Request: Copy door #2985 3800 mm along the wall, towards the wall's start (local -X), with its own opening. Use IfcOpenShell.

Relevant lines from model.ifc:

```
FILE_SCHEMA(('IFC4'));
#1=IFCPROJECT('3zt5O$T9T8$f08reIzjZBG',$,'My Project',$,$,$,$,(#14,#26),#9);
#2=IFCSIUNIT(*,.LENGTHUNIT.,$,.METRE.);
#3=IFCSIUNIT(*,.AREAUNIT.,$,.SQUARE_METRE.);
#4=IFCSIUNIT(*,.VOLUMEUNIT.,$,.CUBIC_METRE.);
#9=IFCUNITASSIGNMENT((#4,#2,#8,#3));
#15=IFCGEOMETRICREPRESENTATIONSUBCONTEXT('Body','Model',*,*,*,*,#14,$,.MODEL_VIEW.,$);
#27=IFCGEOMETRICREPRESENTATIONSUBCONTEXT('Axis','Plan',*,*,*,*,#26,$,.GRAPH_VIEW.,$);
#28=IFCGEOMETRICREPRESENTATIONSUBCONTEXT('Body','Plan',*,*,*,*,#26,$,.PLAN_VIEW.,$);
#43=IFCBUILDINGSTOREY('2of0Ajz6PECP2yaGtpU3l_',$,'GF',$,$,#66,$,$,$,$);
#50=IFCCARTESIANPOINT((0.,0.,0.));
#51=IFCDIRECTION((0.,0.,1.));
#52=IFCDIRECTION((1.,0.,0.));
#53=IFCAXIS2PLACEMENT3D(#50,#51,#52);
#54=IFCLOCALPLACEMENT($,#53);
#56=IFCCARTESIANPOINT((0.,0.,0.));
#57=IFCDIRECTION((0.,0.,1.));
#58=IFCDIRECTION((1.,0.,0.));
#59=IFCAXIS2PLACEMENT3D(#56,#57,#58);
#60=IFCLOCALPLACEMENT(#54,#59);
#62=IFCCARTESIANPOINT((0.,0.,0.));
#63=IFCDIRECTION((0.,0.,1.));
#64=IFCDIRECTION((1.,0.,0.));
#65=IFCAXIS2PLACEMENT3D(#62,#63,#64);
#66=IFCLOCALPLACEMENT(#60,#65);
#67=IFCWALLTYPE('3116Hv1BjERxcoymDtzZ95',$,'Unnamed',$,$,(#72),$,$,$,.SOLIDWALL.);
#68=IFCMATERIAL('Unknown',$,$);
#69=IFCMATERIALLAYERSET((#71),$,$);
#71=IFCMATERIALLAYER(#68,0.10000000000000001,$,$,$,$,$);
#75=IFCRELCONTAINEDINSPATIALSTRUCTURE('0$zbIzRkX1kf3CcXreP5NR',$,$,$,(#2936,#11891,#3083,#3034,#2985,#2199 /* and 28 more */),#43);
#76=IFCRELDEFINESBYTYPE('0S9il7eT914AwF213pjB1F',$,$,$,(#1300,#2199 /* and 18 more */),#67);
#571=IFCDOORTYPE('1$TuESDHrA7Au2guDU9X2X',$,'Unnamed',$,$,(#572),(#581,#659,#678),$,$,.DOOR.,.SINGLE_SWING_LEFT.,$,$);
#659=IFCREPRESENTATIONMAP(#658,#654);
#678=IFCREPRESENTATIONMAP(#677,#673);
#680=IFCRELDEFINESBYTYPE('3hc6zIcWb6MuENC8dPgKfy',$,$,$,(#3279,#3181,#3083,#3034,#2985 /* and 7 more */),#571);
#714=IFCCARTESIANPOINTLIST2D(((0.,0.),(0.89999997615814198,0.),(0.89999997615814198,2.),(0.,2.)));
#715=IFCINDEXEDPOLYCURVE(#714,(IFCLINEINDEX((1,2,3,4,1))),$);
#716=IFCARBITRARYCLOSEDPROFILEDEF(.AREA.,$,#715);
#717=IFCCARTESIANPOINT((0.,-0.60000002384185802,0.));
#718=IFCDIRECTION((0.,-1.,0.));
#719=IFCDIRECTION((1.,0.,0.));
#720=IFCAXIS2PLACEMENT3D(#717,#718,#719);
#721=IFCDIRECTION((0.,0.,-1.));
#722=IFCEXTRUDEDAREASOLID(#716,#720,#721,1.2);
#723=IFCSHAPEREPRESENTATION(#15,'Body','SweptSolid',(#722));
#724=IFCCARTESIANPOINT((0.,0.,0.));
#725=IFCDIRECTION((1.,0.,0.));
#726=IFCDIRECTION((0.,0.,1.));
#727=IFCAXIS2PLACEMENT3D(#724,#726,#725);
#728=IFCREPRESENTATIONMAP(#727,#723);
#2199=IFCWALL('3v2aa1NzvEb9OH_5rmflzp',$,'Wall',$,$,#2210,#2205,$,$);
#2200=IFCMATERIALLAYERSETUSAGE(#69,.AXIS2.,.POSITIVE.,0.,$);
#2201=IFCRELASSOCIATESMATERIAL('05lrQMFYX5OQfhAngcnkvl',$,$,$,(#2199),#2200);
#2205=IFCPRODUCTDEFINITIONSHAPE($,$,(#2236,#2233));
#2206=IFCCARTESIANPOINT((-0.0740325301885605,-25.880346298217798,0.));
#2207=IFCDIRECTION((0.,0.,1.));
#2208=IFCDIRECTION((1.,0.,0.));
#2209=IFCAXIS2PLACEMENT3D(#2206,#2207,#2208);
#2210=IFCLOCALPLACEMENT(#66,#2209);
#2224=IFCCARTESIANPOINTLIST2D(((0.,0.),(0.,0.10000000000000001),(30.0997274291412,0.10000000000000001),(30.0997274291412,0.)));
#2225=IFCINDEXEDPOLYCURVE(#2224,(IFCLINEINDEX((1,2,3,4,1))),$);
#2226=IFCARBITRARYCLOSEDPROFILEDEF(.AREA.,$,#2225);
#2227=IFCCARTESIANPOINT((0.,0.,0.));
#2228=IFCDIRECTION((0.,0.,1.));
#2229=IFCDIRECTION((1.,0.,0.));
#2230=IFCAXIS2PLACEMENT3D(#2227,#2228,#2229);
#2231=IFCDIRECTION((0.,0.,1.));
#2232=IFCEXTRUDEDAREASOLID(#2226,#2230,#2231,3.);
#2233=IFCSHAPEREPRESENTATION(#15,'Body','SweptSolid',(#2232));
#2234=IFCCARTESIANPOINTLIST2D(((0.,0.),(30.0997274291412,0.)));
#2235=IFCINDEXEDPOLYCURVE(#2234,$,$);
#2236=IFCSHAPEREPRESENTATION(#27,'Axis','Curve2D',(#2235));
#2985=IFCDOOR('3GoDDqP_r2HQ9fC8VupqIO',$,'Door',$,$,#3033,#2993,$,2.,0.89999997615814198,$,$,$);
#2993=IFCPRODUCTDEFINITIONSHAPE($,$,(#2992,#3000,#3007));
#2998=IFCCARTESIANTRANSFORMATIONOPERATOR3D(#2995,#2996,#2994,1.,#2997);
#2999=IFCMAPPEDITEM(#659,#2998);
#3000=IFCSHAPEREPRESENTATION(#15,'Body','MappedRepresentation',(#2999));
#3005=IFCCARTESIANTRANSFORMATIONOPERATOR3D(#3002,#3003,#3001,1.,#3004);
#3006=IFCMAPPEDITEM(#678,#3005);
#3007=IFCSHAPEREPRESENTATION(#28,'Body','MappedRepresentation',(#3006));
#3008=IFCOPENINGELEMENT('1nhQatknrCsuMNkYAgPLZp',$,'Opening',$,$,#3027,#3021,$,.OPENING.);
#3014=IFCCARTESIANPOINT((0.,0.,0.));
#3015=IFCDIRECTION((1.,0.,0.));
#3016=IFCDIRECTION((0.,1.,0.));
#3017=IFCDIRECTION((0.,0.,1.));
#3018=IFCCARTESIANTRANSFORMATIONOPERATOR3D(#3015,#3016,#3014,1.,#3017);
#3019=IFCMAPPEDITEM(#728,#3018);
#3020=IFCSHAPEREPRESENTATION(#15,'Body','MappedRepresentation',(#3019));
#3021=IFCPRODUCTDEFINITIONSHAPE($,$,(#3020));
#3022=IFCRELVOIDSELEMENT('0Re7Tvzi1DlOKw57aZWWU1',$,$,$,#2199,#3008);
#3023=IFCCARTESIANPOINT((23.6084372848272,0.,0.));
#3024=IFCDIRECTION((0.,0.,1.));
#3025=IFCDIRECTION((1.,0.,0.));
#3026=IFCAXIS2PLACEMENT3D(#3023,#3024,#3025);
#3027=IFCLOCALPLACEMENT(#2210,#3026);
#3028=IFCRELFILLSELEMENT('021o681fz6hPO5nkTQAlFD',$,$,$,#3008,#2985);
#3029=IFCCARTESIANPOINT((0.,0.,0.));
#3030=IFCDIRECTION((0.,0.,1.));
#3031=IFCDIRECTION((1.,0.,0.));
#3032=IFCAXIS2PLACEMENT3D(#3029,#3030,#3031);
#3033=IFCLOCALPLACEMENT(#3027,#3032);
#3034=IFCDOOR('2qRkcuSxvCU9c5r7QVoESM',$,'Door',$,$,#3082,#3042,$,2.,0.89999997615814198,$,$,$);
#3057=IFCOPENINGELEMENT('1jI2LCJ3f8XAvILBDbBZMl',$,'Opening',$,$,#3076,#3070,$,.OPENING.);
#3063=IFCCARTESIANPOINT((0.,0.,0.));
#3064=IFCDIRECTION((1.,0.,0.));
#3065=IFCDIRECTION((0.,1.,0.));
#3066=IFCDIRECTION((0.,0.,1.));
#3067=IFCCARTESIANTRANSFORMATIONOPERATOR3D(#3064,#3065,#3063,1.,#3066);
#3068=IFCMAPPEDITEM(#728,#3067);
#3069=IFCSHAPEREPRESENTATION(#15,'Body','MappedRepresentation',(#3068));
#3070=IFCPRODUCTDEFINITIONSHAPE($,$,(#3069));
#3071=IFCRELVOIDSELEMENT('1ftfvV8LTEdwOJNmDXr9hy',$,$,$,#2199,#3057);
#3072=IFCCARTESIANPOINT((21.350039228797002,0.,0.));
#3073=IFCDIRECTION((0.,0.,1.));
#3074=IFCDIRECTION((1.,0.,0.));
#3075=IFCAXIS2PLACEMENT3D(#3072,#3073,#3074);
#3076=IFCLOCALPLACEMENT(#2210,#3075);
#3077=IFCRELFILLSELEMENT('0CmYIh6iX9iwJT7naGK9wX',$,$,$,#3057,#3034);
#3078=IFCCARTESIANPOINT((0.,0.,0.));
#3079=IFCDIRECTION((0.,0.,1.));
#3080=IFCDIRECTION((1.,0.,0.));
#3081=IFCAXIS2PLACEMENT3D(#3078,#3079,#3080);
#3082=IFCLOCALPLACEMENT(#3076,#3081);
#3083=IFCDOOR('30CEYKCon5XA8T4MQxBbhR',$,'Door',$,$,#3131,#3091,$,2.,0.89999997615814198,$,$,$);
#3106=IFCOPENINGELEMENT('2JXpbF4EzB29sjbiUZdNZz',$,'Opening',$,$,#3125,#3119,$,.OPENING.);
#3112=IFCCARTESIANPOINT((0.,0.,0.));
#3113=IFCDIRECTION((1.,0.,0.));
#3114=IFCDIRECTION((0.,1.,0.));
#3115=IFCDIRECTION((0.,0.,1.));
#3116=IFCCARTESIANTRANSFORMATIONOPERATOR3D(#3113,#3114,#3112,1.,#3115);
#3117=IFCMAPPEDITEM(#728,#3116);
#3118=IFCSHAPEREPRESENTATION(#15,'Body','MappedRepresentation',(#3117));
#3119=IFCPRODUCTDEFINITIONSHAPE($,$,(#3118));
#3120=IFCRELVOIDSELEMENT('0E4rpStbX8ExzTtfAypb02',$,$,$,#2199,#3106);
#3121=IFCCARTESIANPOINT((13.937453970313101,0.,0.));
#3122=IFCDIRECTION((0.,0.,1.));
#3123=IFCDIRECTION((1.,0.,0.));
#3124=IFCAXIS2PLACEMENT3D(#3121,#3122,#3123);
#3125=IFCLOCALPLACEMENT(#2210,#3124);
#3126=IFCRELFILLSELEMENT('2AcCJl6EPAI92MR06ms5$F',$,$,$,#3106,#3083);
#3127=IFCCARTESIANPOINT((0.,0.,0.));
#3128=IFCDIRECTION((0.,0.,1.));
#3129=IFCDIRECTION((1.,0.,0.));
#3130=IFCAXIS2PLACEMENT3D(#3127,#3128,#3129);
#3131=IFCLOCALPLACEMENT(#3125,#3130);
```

```python
import ifcopenshell
import ifcopenshell.api.feature
import ifcopenshell.api.geometry
import ifcopenshell.api.root
import ifcopenshell.geom
import ifcopenshell.util.element
import ifcopenshell.util.placement
import ifcopenshell.util.shape
import ifcopenshell.util.unit

model = ifcopenshell.open("model.ifc")
unit_scale = ifcopenshell.util.unit.calculate_unit_scale(model)
settings = ifcopenshell.geom.settings()


def volume(element):
    """Net volume in cubic metres, openings subtracted."""
    shape = ifcopenshell.geom.create_shape(settings, element)
    return ifcopenshell.util.shape.get_volume(shape.geometry)


door = model.by_guid("3GoDDqP_r2HQ9fC8VupqIO")
opening = door.FillsVoids[0].RelatingOpeningElement
wall = opening.VoidsElements[0].RelatingBuildingElement
before = volume(wall)
shift = ifcopenshell.util.placement.get_local_placement(wall.ObjectPlacement)[:3, 0] * -3.8 / unit_scale

# copy_class copies the void relationship, type, container and properties, but no geometry.
new_opening = ifcopenshell.api.root.copy_class(model, product=opening)
new_opening.Representation = ifcopenshell.util.element.copy_deep(
    model, opening.Representation, exclude=["IfcGeometricRepresentationContext", "IfcRepresentationMap"]
)
new_door = ifcopenshell.api.root.copy_class(model, product=door)
new_door.Representation = ifcopenshell.util.element.copy_deep(
    model, door.Representation, exclude=["IfcGeometricRepresentationContext", "IfcRepresentationMap"]
)
ifcopenshell.api.feature.add_filling(model, opening=new_opening, element=new_door)

for old, new in ((opening, new_opening), (door, new_door)):
    matrix = ifcopenshell.util.placement.get_local_placement(old.ObjectPlacement)
    matrix[:3, 3] += shift
    ifcopenshell.api.geometry.edit_object_placement(model, product=new, matrix=matrix, is_si=False)

after = volume(wall)

print(f"wall volume {before:.3f} -> {after:.3f} m3")

model.write("model_rev.ifc")
```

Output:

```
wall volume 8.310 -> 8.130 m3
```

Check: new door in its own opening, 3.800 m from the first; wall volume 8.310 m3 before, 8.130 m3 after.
